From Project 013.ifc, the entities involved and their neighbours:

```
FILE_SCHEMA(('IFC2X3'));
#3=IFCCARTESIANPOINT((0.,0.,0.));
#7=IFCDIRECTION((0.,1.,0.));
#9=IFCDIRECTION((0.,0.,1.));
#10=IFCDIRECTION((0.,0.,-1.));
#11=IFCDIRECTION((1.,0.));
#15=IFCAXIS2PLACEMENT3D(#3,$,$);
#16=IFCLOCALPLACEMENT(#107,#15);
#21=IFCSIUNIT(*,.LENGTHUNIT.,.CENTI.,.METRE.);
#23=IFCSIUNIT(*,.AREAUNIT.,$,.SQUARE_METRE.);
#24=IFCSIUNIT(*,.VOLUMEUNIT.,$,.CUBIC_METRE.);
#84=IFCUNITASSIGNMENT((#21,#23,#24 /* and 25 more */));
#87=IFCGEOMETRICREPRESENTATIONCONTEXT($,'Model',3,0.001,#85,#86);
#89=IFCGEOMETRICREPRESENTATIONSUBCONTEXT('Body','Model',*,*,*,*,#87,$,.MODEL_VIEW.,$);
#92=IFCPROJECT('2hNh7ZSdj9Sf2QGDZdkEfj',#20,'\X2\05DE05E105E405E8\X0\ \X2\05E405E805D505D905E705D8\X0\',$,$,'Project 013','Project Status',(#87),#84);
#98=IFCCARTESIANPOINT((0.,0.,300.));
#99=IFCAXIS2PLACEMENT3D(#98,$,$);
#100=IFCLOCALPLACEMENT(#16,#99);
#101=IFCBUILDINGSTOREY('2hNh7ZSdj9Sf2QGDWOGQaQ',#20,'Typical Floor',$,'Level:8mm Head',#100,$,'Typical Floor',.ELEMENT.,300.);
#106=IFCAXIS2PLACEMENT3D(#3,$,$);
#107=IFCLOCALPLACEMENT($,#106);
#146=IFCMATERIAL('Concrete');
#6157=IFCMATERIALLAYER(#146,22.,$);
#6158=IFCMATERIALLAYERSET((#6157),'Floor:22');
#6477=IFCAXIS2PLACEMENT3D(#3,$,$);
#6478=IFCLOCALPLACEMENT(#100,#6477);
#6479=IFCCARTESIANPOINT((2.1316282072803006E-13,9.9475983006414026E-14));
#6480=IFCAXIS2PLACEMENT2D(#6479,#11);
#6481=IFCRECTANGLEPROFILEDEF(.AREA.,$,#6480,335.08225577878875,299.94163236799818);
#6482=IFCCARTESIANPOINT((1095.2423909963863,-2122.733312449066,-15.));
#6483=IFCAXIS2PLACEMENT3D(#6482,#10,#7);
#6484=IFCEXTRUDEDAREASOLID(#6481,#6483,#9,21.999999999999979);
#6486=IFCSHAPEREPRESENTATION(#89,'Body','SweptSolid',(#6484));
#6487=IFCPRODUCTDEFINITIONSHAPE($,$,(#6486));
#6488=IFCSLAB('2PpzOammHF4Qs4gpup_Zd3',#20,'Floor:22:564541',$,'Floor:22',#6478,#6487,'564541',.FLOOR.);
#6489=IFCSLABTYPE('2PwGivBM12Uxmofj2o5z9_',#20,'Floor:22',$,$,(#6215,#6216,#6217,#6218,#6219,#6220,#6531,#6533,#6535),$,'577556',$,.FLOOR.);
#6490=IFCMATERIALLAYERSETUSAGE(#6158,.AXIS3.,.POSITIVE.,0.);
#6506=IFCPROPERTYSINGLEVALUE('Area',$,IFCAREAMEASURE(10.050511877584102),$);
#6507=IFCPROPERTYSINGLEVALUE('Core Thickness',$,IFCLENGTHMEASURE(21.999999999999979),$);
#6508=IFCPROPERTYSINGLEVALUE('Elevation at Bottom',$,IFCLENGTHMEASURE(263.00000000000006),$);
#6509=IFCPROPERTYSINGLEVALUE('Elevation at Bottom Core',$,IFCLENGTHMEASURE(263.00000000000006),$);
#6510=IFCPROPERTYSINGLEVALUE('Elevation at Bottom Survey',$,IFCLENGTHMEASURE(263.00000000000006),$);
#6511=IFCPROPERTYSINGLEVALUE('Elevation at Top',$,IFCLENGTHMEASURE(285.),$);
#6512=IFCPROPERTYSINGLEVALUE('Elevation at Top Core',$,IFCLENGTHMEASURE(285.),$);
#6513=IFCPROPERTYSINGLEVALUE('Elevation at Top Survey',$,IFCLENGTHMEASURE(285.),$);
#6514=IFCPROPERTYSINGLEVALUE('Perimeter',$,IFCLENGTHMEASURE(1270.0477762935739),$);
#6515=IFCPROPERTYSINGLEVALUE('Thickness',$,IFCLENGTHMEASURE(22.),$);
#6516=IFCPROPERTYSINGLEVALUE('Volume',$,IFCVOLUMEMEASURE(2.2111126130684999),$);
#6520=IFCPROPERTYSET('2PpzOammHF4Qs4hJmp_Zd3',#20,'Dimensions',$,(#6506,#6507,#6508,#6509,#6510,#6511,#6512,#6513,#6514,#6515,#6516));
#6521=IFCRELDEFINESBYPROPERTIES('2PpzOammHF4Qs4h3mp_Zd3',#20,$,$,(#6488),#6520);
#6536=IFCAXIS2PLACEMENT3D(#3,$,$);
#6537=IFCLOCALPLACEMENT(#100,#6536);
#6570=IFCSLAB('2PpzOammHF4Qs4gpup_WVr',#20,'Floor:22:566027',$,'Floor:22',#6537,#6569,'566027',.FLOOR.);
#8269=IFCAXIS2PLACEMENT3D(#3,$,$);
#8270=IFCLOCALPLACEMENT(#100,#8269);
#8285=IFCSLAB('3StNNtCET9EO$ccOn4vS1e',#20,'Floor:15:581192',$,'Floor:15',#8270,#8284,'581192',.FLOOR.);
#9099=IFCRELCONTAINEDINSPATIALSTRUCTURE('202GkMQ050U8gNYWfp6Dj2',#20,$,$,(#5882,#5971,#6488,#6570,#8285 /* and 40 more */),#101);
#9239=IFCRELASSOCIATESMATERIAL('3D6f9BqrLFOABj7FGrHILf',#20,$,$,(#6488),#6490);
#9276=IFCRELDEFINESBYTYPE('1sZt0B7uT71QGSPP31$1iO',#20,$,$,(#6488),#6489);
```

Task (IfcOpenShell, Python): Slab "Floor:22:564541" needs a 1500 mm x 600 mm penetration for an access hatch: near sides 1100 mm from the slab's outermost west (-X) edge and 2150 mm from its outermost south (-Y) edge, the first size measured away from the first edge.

```python
import numpy as np
import ifcopenshell
import ifcopenshell.api.feature
import ifcopenshell.api.geometry
import ifcopenshell.api.pset
import ifcopenshell.api.root
import ifcopenshell.geom
import ifcopenshell.util.element
import ifcopenshell.util.placement
import ifcopenshell.util.representation
import ifcopenshell.util.shape
import ifcopenshell.util.unit

model = ifcopenshell.open("Project 013.ifc")
unit_scale = ifcopenshell.util.unit.calculate_unit_scale(model)
area_scale = ifcopenshell.util.unit.calculate_unit_scale(model, "AREAUNIT")
volume_scale = ifcopenshell.util.unit.calculate_unit_scale(model, "VOLUMEUNIT")
settings = ifcopenshell.geom.settings()


def volume(element):
    """Net volume in cubic metres, openings subtracted."""
    shape = ifcopenshell.geom.create_shape(settings, element)
    return ifcopenshell.util.shape.get_volume(shape.geometry)


slab = model.by_id(6488)
before = volume(slab)

# Extent in the slab's own axes, in metres. The edges named are its -X and -Y sides.
slab_shape = ifcopenshell.geom.create_shape(settings, slab)
vertices = ifcopenshell.util.shape.get_vertices(slab_shape.geometry)
x_min, y_min, bottom = vertices.min(axis=0)
top = vertices[:, 2].max()

opening = ifcopenshell.api.root.create_entity(model, ifc_class="IfcOpeningElement", name="Access hatch opening")
context = ifcopenshell.util.representation.get_context(model, "Model", "Body", "MODEL_VIEW")
width, depth = 1.5, 0.6
outline = [(0.0, 0.0), (width, 0.0), (width, depth), (0.0, depth), (0.0, 0.0)]
# Overshoot both faces by 50 mm so the cut is clean.
shape = ifcopenshell.api.geometry.add_slab_representation(
    model, context=context, depth=top - bottom + 0.1, polyline=outline
)
ifcopenshell.api.geometry.assign_representation(model, product=opening, representation=shape)

matrix = ifcopenshell.util.placement.get_local_placement(slab.ObjectPlacement)
matrix[:, 3] = matrix @ np.append(np.array([x_min + 1.1, y_min + 2.15, bottom - 0.05]) / unit_scale, 1.0)
ifcopenshell.api.geometry.edit_object_placement(model, product=opening, matrix=matrix, is_si=False)
ifcopenshell.api.feature.add_feature(model, feature=opening, element=slab)

after = volume(slab)

# Update the slab's stored quantities.
pset = model.by_id(ifcopenshell.util.element.get_pset(slab, "Dimensions", should_inherit=False)["id"])
ifcopenshell.api.pset.edit_pset(model, pset=pset, properties={
    "Area": model.create_entity("IfcAreaMeasure", after / (top - bottom) / area_scale),
    "Volume": model.create_entity("IfcVolumeMeasure", after / volume_scale),
})

print(f"slab volume {before:.3f} -> {after:.3f} m3")

model.write("Project 013_rev.ifc")
```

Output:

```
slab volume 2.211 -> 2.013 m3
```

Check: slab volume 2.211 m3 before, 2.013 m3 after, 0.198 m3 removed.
